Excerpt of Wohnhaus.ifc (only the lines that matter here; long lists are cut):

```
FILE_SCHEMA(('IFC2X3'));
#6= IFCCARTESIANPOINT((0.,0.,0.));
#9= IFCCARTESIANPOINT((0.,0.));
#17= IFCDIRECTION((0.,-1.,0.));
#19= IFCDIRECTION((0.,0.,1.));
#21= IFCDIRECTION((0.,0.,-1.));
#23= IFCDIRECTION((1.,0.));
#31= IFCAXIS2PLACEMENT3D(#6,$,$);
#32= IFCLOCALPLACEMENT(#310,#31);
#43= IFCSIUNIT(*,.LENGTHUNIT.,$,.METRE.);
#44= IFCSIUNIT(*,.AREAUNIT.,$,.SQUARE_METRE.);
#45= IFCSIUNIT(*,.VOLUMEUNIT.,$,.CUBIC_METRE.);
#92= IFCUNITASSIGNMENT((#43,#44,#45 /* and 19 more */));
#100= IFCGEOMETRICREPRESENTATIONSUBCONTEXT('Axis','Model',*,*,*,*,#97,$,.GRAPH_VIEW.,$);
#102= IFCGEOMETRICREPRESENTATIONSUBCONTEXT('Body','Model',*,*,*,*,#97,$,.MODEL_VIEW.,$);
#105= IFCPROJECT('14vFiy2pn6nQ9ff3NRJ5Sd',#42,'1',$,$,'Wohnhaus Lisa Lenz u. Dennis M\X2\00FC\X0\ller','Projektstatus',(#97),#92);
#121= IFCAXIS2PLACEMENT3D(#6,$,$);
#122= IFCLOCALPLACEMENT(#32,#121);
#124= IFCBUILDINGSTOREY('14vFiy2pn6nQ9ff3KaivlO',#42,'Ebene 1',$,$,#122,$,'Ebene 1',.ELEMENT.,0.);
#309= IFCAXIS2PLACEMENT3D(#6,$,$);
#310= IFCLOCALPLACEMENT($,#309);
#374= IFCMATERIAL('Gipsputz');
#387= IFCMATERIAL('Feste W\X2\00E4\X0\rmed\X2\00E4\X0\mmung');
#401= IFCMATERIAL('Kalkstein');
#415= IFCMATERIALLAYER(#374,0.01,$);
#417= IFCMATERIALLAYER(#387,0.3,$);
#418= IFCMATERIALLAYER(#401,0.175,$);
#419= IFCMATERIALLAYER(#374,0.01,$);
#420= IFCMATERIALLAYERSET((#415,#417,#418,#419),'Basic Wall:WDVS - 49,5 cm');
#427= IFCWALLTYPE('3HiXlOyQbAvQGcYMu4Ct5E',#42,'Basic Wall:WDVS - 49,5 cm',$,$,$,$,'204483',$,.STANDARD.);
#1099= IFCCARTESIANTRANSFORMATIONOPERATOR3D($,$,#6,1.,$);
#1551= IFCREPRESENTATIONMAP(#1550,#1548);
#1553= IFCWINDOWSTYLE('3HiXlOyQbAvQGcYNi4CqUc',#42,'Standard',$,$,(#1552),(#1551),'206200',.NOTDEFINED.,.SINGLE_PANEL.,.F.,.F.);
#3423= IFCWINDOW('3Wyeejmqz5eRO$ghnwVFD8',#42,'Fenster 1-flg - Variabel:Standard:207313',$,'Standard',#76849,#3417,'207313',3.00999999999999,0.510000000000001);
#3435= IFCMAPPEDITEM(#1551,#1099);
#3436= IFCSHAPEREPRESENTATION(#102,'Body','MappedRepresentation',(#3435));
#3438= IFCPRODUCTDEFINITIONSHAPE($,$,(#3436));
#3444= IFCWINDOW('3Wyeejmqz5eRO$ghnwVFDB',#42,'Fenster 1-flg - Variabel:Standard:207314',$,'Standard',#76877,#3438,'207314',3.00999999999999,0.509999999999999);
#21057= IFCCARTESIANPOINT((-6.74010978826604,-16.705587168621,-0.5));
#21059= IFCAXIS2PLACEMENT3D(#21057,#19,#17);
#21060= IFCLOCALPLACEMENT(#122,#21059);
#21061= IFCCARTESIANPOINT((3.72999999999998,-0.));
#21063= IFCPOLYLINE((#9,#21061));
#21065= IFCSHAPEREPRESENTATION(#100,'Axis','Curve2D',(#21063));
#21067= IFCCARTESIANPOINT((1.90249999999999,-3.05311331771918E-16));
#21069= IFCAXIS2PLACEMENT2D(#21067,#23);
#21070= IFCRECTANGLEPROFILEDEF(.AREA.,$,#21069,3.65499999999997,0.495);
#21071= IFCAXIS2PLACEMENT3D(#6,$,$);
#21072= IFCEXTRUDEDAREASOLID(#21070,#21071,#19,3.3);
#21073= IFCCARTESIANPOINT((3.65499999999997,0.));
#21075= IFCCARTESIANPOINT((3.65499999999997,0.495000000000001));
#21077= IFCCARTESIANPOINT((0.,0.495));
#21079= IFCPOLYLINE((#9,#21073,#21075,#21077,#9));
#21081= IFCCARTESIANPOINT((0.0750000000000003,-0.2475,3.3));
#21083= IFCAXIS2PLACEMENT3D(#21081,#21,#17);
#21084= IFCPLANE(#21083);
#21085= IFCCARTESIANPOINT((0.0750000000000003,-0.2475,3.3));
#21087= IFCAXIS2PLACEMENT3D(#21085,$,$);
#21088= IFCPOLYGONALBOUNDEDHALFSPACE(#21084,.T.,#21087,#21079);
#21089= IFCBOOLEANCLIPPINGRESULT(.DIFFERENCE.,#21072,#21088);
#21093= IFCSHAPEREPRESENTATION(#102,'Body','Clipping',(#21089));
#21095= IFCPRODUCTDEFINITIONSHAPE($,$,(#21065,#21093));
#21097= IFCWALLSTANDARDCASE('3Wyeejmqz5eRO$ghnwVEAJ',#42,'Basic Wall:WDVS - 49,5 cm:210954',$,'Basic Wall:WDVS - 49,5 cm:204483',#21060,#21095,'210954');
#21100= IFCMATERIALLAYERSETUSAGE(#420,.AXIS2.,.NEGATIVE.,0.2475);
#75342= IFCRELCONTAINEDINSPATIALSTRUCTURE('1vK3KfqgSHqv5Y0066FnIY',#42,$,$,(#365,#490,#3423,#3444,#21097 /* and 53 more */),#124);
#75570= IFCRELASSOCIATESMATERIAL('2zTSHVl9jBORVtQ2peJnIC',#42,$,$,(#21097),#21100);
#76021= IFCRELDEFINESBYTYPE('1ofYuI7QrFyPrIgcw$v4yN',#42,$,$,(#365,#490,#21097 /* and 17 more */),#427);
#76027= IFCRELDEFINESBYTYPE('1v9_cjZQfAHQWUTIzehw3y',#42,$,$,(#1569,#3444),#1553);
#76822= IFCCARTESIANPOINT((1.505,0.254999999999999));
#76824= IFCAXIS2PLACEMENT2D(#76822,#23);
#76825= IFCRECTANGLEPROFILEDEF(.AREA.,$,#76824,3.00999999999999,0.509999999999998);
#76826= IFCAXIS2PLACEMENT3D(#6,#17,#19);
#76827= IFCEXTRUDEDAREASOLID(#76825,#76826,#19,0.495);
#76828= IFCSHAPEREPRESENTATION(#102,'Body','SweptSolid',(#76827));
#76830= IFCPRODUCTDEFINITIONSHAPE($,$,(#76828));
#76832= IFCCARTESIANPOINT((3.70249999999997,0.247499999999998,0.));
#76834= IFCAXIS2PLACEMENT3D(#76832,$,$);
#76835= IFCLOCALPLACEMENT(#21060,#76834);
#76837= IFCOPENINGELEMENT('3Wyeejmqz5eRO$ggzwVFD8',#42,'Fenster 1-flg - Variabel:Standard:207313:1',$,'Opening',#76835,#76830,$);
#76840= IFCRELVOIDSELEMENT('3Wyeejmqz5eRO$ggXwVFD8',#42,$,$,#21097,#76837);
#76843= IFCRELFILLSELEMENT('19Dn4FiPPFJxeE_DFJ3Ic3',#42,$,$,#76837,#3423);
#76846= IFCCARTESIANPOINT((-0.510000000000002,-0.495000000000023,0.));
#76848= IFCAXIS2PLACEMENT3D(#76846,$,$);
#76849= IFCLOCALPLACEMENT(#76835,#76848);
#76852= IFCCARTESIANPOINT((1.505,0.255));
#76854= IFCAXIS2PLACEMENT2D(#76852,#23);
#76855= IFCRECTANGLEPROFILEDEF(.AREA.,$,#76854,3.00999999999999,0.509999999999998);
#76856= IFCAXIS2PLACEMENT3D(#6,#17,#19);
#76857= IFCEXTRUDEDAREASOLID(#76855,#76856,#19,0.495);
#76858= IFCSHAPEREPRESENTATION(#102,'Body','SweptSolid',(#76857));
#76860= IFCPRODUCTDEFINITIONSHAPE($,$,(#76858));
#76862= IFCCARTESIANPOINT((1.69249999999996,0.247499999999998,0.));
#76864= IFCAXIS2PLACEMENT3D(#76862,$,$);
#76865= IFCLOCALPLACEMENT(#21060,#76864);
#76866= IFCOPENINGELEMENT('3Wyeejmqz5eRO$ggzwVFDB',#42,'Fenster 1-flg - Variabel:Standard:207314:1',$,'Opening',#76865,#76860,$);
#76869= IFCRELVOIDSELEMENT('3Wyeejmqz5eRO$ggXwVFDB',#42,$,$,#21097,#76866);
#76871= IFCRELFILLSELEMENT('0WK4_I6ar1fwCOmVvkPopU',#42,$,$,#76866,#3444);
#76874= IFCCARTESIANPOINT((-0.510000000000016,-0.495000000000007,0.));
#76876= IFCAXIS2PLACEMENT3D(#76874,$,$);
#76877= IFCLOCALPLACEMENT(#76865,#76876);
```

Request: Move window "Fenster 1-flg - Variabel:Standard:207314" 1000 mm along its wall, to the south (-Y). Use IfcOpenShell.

```python
import ifcopenshell
import ifcopenshell.api.geometry
import ifcopenshell.util.placement

model = ifcopenshell.open("Wohnhaus.ifc")

window = model.by_guid("3Wyeejmqz5eRO$ghnwVFDB")
opening = window.FillsVoids[0].RelatingOpeningElement
wall = opening.VoidsElements[0].RelatingBuildingElement

wall_matrix = ifcopenshell.util.placement.get_local_placement(wall.ObjectPlacement)
shift = wall_matrix[:3, 0] * 1.0
before = ifcopenshell.util.placement.get_local_placement(window.ObjectPlacement)[:3, 3].copy()

# The window is placed relative to its opening, so it follows when the opening moves.
matrix = ifcopenshell.util.placement.get_local_placement(opening.ObjectPlacement)
matrix[:3, 3] += shift
ifcopenshell.api.geometry.edit_object_placement(
    model, product=opening, matrix=matrix, is_si=False, should_transform_children=True
)

after = ifcopenshell.util.placement.get_local_placement(window.ObjectPlacement)[:3, 3]
print("window moved by", (after - before).round(3) + 0.0)

model.write("Wohnhaus_edited.ifc")
```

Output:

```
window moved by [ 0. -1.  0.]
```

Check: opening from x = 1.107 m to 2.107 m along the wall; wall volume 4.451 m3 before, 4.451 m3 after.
